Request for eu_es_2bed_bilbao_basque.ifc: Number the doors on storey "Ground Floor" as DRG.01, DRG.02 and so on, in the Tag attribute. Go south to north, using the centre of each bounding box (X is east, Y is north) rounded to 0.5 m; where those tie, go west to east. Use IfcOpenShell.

First a look at what the model holds.

```python
import ifcopenshell
import ifcopenshell.util.element
import ifcopenshell.util.placement

model = ifcopenshell.open("eu_es_2bed_bilbao_basque.ifc")
print(model.schema)
storey = next(s for s in model.by_type("IfcBuildingStorey") if s.Name == "Ground Floor")
doors = [e for e in ifcopenshell.util.element.get_decomposition(storey) if e.is_a("IfcDoor")]
for e in sorted(doors, key=lambda e: e.id()):
    origin = ifcopenshell.util.placement.get_local_placement(e.ObjectPlacement)[:3, 3]
    print(e.id(), e.Tag, e.Name, origin.round(2) + 0.0, sep=" | ")
```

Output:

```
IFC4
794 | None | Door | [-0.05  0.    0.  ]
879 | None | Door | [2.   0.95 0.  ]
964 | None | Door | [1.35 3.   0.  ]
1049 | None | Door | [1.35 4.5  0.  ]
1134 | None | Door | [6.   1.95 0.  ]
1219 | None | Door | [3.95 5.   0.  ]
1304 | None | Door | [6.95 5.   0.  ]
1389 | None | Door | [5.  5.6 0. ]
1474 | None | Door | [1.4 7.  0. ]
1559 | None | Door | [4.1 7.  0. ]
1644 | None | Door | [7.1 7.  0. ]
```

```python
import ifcopenshell
import ifcopenshell.geom
import ifcopenshell.util.element
import ifcopenshell.util.shape

model = ifcopenshell.open("eu_es_2bed_bilbao_basque.ifc")
settings = ifcopenshell.geom.settings()
settings.set("use-world-coords", True)


def centre(element):
    shape = ifcopenshell.geom.create_shape(settings, element)
    return ifcopenshell.util.shape.get_bbox_centroid(shape.geometry)


storey = next(s for s in model.by_type("IfcBuildingStorey") if s.Name == "Ground Floor")
doors = [e for e in ifcopenshell.util.element.get_decomposition(storey) if e.is_a("IfcDoor")]

# Insertion points can sit at a corner or the storey origin, so sort by the geometry (in metres).
centres = {e: centre(e) for e in doors}
doors.sort(key=lambda e: (round(centres[e][1] / 0.5), centres[e][0]))

for i, e in enumerate(doors, start=1):
    number = f"DRG.{i:02d}"
    e.Tag = number
    print(e.id(), number)

model.write("eu_es_2bed_bilbao_basque_rev.ifc")
```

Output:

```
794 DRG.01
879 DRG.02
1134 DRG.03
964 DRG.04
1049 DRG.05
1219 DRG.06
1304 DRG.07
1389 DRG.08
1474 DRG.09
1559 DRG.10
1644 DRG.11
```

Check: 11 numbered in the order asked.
